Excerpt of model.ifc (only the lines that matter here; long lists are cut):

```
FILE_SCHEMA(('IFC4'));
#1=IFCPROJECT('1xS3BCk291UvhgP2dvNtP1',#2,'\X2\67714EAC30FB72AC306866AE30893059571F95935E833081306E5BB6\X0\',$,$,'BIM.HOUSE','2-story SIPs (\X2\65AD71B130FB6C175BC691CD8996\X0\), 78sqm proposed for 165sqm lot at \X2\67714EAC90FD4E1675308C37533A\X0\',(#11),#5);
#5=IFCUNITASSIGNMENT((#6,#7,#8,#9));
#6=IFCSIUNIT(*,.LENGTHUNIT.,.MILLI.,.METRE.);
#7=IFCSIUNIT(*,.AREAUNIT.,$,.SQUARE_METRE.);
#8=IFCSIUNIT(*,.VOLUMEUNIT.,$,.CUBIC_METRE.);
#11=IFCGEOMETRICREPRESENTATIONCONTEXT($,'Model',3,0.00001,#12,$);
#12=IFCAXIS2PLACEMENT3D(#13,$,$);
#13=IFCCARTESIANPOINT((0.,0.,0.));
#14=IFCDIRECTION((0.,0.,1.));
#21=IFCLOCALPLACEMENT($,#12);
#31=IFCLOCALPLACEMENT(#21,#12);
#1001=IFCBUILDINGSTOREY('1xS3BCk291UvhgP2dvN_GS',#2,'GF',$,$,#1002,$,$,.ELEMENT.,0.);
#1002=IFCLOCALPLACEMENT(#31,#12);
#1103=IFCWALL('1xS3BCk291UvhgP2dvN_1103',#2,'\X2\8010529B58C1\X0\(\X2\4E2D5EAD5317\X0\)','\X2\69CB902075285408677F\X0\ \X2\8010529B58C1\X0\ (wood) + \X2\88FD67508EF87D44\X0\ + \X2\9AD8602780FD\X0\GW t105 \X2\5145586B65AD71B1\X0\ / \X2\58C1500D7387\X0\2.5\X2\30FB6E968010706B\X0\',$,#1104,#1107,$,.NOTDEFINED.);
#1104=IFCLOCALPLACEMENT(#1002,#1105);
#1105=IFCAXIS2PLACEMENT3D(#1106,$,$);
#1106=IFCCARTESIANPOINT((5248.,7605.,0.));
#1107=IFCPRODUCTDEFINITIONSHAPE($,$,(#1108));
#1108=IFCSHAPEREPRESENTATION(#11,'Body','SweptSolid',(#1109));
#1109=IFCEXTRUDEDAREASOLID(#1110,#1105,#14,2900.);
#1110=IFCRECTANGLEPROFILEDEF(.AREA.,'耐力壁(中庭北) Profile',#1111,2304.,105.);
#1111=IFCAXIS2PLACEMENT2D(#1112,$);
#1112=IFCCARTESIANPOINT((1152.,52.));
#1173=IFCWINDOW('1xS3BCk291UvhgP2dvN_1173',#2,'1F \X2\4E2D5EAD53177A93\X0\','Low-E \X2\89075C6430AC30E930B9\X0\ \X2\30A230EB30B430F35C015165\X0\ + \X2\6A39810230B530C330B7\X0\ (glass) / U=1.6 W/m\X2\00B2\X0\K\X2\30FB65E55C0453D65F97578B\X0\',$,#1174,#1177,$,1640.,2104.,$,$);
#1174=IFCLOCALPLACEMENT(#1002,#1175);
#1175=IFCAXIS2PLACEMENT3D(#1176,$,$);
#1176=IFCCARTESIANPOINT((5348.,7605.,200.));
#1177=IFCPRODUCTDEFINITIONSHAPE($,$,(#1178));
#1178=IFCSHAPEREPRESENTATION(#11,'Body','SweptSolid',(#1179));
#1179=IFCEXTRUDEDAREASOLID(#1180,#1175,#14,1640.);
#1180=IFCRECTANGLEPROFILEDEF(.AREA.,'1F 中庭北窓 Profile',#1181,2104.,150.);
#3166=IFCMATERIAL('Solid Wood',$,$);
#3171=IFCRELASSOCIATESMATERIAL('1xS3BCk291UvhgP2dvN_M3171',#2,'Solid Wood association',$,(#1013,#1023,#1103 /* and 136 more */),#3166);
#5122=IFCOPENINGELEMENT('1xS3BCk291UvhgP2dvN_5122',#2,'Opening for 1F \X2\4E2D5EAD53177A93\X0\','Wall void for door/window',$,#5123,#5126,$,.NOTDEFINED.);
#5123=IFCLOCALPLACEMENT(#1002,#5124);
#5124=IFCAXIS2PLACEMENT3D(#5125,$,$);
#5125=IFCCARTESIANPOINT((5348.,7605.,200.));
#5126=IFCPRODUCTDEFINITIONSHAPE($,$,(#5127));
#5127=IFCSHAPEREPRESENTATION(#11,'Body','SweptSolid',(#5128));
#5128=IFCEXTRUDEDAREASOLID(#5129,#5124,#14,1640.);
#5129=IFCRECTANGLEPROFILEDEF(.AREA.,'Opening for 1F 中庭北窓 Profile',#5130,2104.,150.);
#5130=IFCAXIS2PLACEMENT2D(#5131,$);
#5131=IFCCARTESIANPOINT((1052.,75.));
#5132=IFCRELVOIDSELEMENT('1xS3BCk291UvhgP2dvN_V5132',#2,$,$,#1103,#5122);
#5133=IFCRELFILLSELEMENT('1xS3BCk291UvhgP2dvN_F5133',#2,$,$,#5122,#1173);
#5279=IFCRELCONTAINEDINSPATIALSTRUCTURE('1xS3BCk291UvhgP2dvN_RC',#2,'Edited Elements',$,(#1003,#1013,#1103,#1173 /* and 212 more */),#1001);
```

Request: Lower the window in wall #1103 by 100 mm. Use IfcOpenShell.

```python
import numpy as np
import ifcopenshell
import ifcopenshell.api.geometry
import ifcopenshell.util.placement
import ifcopenshell.util.unit

model = ifcopenshell.open("model.ifc")
unit_scale = ifcopenshell.util.unit.calculate_unit_scale(model)

window = model.by_id(1173)
opening = window.FillsVoids[0].RelatingOpeningElement
dz = -0.1 / unit_scale

shift = np.array([0.0, 0.0, dz])
# The window is not placed relative to its opening, so move both.
for product in (opening, window):
    matrix = ifcopenshell.util.placement.get_local_placement(product.ObjectPlacement)
    matrix[:3, 3] += shift
    ifcopenshell.api.geometry.edit_object_placement(model, product=product, matrix=matrix, is_si=False)

print(f"moved by {dz * unit_scale:+.3f} m")

model.write("model_updated.ifc")
```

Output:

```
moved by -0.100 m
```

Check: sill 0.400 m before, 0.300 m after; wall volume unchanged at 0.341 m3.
